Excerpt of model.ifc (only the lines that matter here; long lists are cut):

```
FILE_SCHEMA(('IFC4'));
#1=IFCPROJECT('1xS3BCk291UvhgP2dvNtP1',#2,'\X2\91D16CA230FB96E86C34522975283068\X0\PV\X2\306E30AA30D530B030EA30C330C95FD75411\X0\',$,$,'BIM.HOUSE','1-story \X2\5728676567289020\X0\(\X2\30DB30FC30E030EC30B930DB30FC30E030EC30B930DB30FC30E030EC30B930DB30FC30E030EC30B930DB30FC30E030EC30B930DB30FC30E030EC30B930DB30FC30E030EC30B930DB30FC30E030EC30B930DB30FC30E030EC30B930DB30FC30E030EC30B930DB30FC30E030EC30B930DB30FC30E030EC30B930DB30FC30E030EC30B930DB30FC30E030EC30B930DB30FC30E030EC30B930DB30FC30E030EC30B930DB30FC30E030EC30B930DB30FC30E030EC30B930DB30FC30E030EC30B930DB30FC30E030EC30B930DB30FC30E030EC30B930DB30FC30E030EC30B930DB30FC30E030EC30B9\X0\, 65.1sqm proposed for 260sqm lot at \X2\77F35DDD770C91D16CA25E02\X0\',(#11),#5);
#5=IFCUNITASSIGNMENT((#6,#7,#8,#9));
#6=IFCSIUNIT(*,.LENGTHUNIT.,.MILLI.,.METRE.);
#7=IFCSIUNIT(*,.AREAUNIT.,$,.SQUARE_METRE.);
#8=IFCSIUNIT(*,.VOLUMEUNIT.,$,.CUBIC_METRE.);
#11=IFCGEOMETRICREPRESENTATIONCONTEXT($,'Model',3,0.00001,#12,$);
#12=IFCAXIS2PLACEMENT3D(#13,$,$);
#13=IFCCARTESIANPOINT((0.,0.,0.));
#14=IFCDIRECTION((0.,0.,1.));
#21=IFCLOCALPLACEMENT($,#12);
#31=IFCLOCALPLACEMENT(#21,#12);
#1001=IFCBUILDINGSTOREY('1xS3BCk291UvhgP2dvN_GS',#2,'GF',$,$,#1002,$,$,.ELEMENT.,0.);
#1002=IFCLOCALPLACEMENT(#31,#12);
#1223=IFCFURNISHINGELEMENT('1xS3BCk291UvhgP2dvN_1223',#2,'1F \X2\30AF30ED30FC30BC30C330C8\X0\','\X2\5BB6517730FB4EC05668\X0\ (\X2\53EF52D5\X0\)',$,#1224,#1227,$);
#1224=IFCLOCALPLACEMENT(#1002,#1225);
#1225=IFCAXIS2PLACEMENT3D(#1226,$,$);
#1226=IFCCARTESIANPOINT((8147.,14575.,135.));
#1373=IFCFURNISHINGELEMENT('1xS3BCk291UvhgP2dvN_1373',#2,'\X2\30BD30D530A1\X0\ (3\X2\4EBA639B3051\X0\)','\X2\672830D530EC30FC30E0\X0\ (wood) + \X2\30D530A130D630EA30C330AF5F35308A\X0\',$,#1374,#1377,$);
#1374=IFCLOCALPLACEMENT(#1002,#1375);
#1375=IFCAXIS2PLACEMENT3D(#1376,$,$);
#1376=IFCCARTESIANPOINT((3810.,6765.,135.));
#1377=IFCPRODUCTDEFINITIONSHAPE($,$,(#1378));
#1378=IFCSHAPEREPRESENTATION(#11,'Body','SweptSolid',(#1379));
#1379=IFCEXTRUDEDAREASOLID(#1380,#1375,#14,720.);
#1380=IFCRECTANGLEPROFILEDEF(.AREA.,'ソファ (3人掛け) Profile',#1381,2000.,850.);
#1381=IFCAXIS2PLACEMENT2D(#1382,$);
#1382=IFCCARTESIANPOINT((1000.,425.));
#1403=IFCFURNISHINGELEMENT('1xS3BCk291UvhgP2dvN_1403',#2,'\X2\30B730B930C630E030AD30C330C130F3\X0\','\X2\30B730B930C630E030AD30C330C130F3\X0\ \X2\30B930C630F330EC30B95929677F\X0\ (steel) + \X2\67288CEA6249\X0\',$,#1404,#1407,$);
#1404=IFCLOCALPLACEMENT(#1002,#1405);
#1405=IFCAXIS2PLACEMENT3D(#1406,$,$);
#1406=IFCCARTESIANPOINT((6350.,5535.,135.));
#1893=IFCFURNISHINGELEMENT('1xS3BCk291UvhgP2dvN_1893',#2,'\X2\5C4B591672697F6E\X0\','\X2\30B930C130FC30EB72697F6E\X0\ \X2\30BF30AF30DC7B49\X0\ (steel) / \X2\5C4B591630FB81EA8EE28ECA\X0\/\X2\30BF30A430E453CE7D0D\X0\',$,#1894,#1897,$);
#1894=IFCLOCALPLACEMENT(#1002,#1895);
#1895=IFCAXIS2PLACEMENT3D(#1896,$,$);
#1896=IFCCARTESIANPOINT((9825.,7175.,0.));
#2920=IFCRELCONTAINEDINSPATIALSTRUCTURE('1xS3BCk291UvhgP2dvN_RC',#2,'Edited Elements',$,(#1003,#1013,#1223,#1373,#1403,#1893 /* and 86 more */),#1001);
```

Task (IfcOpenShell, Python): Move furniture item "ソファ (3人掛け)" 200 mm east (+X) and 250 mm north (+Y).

```python
import ifcopenshell
import ifcopenshell.api.geometry
import ifcopenshell.util.placement
import ifcopenshell.util.unit

model = ifcopenshell.open("model.ifc")
unit_scale = ifcopenshell.util.unit.calculate_unit_scale(model)

item = model.by_guid("1xS3BCk291UvhgP2dvN_1373")
matrix = ifcopenshell.util.placement.get_local_placement(item.ObjectPlacement)
matrix[0, 3] += 0.2 / unit_scale
matrix[1, 3] += 0.25 / unit_scale
ifcopenshell.api.geometry.edit_object_placement(model, product=item, matrix=matrix, is_si=False)

print(ifcopenshell.util.placement.get_local_placement(item.ObjectPlacement).round(3) + 0.0)

model.write("model_v2.ifc")
```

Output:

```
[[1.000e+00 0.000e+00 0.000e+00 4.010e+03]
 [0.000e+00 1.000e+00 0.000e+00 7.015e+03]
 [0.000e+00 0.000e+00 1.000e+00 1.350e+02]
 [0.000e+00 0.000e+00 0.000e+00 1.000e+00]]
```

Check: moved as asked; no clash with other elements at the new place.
